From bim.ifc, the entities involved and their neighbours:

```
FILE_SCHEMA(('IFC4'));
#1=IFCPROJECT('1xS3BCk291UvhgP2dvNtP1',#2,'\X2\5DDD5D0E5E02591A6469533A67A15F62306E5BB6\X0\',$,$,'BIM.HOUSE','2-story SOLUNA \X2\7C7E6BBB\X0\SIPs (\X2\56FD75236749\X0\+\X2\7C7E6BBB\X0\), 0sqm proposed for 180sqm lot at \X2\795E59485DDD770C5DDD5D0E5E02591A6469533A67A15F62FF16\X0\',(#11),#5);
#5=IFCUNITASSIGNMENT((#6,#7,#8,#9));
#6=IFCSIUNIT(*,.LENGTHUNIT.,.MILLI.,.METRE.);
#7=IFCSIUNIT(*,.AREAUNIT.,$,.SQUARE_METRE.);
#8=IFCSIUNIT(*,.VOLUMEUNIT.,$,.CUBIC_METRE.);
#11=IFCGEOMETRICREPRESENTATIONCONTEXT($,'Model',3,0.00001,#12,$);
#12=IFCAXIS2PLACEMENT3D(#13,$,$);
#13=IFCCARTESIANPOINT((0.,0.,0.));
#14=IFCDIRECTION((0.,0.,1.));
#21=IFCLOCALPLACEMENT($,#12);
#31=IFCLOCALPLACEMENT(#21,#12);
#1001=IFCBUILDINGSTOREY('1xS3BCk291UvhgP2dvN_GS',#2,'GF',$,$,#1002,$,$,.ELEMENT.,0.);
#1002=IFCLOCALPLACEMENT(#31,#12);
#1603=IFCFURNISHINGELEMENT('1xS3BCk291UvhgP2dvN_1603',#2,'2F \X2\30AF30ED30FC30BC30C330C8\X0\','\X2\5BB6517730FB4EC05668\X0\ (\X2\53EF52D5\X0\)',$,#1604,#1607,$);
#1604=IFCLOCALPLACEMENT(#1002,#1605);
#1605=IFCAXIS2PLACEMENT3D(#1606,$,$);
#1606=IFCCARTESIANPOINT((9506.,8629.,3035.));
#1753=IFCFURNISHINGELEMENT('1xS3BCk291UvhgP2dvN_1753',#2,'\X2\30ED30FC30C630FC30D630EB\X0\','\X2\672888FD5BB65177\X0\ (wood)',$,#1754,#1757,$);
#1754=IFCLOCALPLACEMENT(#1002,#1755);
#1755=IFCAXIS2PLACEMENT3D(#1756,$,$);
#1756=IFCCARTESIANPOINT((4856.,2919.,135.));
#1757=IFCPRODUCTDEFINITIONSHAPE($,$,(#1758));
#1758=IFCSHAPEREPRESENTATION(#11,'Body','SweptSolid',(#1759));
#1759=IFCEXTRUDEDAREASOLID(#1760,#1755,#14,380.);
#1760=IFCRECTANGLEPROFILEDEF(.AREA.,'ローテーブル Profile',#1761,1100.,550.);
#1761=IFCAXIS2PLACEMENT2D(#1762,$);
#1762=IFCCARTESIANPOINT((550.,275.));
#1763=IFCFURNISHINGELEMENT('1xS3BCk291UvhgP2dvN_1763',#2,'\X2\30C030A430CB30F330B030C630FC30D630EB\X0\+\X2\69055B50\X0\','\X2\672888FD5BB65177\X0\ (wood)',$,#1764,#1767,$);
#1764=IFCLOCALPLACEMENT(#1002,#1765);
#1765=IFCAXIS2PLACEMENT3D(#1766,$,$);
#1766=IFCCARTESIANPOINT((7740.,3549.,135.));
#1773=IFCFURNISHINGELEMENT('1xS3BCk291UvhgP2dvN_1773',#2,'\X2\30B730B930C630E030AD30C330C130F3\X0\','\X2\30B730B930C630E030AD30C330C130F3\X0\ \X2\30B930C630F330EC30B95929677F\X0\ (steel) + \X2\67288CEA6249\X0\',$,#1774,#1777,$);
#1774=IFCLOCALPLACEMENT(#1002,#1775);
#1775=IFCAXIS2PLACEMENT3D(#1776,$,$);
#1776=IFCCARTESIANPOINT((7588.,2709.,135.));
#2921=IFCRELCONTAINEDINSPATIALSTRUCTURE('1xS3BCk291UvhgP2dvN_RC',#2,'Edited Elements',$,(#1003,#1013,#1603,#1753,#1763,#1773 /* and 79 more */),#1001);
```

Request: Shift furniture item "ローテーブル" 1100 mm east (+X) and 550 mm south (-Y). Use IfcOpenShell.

```python
import ifcopenshell
import ifcopenshell.api.geometry
import ifcopenshell.util.placement

model = ifcopenshell.open("bim.ifc")

item = model.by_guid("1xS3BCk291UvhgP2dvN_1753")
matrix = ifcopenshell.util.placement.get_local_placement(item.ObjectPlacement)
matrix[0, 3] += 1100.0
matrix[1, 3] -= 550.0
ifcopenshell.api.geometry.edit_object_placement(model, product=item, matrix=matrix, is_si=False)

print(ifcopenshell.util.placement.get_local_placement(item.ObjectPlacement).round(3) + 0.0)

model.write("bim_v2.ifc")
```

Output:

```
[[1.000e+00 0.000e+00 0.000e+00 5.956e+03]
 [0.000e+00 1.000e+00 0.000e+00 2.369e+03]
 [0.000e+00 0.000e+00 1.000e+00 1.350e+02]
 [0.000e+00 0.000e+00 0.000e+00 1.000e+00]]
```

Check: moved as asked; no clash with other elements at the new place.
